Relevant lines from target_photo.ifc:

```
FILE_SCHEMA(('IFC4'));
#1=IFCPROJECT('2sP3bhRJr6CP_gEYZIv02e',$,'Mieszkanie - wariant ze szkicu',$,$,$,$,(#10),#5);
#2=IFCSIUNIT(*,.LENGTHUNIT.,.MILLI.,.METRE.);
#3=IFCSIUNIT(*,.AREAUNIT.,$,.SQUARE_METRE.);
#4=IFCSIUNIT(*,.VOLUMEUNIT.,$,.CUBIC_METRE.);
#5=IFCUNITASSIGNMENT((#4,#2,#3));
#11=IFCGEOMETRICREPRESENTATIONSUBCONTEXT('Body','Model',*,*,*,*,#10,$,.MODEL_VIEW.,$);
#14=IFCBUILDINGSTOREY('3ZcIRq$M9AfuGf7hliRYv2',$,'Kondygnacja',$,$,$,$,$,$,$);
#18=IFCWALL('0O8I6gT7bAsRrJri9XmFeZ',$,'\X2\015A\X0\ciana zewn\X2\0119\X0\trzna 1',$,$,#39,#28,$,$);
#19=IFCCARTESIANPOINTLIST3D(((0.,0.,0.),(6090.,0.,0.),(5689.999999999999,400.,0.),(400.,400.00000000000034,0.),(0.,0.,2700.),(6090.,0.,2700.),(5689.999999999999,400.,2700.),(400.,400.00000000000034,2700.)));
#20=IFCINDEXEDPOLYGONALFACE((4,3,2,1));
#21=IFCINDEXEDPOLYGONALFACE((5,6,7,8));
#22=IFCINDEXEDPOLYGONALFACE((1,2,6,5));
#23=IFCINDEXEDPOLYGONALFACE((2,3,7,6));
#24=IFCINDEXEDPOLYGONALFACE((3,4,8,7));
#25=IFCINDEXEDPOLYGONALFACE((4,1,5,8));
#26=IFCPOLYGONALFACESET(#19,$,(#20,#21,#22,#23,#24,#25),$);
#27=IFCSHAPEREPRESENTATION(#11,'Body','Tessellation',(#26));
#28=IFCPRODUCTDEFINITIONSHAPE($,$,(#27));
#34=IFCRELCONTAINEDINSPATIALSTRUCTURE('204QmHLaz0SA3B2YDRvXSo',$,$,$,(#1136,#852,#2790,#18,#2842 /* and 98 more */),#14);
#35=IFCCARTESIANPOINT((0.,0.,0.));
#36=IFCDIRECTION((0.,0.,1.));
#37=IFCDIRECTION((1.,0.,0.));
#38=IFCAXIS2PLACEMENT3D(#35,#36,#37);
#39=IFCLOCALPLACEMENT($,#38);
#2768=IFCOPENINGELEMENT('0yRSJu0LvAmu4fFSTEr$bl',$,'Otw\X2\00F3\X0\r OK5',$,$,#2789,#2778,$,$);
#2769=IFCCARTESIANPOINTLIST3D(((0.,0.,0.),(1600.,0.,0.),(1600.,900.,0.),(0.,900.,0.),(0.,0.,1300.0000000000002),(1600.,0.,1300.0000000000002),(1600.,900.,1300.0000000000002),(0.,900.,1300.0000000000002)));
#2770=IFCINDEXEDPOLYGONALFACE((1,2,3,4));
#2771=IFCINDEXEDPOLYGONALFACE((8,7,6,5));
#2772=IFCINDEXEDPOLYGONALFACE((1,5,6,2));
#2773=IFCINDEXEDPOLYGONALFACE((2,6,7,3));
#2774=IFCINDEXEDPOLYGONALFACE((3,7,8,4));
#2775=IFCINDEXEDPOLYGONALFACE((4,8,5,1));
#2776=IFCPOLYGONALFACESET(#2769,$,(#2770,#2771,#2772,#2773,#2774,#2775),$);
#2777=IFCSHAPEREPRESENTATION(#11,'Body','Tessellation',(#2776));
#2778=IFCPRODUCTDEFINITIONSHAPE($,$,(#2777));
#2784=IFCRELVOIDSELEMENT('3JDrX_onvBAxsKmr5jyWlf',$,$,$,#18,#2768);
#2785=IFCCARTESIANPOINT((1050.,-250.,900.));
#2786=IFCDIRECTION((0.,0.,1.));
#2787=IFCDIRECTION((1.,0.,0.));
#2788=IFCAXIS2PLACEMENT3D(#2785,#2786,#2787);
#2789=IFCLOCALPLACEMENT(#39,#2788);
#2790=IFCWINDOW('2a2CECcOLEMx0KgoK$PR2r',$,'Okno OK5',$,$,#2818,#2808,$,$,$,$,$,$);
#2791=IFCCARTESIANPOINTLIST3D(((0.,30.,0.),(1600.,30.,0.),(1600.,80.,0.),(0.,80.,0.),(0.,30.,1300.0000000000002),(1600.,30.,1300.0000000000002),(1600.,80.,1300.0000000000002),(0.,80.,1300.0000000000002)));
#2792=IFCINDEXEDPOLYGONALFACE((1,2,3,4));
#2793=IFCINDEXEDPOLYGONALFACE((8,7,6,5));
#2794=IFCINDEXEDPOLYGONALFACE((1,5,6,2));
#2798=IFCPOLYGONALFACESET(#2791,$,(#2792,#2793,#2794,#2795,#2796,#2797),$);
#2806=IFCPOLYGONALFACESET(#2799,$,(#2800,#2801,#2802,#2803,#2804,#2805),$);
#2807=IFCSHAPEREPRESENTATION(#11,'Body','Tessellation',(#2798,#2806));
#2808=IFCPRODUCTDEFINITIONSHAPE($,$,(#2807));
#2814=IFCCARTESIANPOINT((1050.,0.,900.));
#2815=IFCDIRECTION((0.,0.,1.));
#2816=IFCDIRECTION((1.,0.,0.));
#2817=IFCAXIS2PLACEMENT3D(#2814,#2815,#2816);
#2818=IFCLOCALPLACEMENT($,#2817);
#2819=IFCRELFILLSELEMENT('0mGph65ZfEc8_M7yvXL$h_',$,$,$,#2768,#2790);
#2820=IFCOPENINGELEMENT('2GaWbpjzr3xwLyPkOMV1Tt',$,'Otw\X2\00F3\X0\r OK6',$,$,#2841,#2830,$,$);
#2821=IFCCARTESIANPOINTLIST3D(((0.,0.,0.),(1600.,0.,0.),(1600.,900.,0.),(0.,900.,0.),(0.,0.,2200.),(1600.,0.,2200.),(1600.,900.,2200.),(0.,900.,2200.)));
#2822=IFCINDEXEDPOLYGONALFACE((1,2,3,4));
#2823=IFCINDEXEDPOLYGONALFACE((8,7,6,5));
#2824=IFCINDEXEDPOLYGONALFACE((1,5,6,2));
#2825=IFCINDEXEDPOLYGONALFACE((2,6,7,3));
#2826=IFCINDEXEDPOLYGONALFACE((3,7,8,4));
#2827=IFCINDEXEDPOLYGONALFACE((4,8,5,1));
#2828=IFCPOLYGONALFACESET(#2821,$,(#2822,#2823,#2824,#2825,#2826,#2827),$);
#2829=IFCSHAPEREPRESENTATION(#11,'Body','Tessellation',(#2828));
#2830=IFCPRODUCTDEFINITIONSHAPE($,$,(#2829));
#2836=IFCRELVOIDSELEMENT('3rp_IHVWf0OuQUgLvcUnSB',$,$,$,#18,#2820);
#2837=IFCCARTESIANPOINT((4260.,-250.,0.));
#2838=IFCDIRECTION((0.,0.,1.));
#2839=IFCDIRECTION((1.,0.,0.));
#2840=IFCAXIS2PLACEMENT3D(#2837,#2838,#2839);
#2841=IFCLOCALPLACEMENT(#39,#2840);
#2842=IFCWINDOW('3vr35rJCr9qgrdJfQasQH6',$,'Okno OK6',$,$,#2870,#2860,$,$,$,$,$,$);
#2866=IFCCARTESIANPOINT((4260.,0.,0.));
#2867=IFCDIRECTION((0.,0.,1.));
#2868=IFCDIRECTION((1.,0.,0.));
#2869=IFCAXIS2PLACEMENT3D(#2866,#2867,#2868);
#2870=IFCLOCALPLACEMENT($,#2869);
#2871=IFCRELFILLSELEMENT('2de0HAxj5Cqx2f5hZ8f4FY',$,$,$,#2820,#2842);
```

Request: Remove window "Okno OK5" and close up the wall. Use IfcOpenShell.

```python
import ifcopenshell
import ifcopenshell.api.feature
import ifcopenshell.api.root
import ifcopenshell.geom
import ifcopenshell.util.shape

model = ifcopenshell.open("target_photo.ifc")
settings = ifcopenshell.geom.settings()


def volume(element):
    """Net volume in cubic metres, openings subtracted."""
    shape = ifcopenshell.geom.create_shape(settings, element)
    return ifcopenshell.util.shape.get_volume(shape.geometry)


window = model.by_id(2790)
opening = window.FillsVoids[0].RelatingOpeningElement
wall = opening.VoidsElements[0].RelatingBuildingElement
before = volume(wall)

ifcopenshell.api.root.remove_product(model, product=window)
ifcopenshell.api.feature.remove_feature(model, feature=opening)

after = volume(wall)

print(f"wall volume {before:.3f} -> {after:.3f} m3")

model.write("target_photo-out.ifc")
```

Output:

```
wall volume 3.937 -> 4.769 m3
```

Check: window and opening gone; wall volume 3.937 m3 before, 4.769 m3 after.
